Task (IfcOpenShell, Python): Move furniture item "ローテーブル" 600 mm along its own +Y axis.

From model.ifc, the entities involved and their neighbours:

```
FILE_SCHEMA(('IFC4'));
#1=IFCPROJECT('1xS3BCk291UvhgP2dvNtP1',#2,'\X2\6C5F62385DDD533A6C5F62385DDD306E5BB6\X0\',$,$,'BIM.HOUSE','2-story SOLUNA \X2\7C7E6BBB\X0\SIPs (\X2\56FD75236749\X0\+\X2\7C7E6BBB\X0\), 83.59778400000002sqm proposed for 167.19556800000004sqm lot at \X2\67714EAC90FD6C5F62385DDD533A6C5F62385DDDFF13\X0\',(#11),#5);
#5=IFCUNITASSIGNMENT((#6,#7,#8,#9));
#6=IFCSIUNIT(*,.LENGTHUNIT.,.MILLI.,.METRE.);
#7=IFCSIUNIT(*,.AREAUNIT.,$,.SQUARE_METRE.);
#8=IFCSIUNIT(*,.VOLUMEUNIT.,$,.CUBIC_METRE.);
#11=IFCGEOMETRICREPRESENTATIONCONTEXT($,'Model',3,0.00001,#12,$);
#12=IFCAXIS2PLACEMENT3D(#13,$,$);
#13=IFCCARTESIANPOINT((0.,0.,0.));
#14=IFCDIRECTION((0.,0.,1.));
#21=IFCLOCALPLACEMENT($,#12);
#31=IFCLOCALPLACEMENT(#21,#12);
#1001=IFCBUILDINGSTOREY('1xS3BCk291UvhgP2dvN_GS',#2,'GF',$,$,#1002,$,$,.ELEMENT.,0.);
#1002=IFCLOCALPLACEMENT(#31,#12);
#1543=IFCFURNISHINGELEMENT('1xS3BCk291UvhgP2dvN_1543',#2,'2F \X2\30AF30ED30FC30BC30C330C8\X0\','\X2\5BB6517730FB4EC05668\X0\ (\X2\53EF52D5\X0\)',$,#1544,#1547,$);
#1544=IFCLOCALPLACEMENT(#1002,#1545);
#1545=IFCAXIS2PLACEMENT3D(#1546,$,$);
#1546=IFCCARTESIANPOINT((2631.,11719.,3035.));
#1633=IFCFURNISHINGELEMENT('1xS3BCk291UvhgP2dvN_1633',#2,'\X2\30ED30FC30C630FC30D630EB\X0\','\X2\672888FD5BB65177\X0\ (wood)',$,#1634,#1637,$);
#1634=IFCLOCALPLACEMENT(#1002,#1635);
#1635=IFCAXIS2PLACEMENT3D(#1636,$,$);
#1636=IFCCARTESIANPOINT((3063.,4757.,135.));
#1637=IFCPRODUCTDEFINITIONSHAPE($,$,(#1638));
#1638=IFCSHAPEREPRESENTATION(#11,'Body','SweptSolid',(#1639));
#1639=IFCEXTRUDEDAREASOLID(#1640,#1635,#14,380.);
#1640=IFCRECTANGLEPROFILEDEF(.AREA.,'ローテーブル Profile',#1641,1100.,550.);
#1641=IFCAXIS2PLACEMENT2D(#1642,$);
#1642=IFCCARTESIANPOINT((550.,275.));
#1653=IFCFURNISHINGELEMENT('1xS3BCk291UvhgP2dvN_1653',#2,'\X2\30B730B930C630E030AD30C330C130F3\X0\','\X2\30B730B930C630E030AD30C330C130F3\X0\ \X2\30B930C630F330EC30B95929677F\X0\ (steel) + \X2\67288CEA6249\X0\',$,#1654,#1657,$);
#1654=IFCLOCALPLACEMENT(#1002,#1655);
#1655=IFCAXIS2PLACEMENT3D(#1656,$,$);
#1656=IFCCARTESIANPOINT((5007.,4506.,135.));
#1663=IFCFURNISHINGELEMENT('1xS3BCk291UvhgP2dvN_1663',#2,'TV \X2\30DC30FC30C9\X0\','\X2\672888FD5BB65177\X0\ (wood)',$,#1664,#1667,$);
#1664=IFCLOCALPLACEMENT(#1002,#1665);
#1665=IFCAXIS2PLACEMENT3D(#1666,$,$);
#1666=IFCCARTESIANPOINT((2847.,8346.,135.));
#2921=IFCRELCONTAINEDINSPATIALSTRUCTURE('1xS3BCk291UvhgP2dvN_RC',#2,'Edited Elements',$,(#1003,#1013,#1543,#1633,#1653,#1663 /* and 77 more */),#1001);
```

```python
import ifcopenshell
import ifcopenshell.api.geometry
import ifcopenshell.util.placement
import ifcopenshell.util.unit

model = ifcopenshell.open("model.ifc")
unit_scale = ifcopenshell.util.unit.calculate_unit_scale(model)

item = model.by_guid("1xS3BCk291UvhgP2dvN_1633")
matrix = ifcopenshell.util.placement.get_local_placement(item.ObjectPlacement)
matrix[:3, 3] += matrix[:3, 1] * 0.6 / unit_scale
ifcopenshell.api.geometry.edit_object_placement(model, product=item, matrix=matrix, is_si=False)

print(ifcopenshell.util.placement.get_local_placement(item.ObjectPlacement).round(3) + 0.0)

model.write("model_edited.ifc")
```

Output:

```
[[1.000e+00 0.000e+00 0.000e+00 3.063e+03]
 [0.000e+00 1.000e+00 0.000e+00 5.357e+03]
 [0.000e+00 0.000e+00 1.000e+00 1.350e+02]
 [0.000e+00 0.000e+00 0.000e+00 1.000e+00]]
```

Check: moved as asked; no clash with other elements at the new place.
